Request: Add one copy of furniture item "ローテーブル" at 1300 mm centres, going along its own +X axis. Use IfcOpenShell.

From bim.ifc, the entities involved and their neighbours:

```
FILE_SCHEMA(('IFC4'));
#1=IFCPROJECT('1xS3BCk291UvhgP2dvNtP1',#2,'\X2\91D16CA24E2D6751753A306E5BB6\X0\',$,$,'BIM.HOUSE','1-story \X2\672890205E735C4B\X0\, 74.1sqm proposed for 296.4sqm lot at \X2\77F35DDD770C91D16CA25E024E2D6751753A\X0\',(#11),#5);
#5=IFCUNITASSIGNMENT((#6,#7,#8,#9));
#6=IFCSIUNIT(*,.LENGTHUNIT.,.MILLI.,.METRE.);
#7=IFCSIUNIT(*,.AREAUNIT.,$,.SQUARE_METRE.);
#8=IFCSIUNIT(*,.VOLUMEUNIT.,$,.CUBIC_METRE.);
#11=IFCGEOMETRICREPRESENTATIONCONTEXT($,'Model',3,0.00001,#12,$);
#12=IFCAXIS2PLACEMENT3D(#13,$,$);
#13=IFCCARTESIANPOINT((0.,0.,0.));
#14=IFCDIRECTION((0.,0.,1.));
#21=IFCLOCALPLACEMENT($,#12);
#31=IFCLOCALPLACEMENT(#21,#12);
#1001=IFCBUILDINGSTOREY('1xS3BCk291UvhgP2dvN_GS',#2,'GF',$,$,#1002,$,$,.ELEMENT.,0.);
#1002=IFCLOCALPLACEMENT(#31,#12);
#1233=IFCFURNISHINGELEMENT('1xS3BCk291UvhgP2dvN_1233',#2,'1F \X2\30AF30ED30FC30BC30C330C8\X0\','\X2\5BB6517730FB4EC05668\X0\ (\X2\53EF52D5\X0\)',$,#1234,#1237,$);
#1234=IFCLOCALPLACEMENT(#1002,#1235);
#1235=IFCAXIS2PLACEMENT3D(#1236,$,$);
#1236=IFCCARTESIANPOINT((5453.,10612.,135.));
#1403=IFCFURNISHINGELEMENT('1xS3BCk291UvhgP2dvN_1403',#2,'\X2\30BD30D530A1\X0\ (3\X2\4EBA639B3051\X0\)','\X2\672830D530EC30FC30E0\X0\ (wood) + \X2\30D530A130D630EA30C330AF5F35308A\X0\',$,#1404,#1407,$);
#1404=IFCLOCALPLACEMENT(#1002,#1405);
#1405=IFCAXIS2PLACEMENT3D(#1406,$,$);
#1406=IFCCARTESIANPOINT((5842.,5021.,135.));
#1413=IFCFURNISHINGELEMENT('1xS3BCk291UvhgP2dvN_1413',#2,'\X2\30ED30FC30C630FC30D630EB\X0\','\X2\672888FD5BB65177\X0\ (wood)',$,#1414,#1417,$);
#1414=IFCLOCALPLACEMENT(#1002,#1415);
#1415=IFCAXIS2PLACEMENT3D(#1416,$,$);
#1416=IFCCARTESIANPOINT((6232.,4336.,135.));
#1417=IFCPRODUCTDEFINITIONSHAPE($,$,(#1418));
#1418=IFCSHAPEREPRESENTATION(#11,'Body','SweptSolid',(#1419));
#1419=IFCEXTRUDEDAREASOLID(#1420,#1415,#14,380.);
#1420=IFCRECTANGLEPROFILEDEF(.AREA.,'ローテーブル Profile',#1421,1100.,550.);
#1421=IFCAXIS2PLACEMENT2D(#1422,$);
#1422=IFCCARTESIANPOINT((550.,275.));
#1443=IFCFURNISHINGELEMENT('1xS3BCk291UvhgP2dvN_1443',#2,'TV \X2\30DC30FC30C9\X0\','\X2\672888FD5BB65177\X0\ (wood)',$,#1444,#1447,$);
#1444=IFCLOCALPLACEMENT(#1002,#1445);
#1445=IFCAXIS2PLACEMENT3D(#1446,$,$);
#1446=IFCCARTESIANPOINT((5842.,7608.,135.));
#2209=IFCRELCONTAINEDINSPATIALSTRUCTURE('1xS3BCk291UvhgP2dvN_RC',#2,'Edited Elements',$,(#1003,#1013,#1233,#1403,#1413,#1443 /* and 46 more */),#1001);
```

```python
import ifcopenshell
import ifcopenshell.api.geometry
import ifcopenshell.api.root
import ifcopenshell.util.element
import ifcopenshell.util.placement
import ifcopenshell.util.unit

model = ifcopenshell.open("bim.ifc")
unit_scale = ifcopenshell.util.unit.calculate_unit_scale(model)


def reuse_history(source, copy):
    """copy_class also copies each property set's owner history, people and application; keep the originals."""
    for rel in copy.IsDefinedBy:
        if rel.is_a("IfcRelDefinesByProperties") and (history := rel.RelatingPropertyDefinition.OwnerHistory):
            rel.RelatingPropertyDefinition.OwnerHistory = source.OwnerHistory
            ifcopenshell.util.element.remove_deep2(model, history)


source = model.by_guid("1xS3BCk291UvhgP2dvN_1413")
base = ifcopenshell.util.placement.get_local_placement(source.ObjectPlacement)
step = base[:3, 0] * 1.3 / unit_scale

for i in range(1, 2):
    copy = ifcopenshell.api.root.copy_class(model, product=source)
    copy.Representation = ifcopenshell.util.element.copy_deep(
        model, source.Representation, exclude=["IfcGeometricRepresentationContext", "IfcRepresentationMap"]
    )
    reuse_history(source, copy)
    matrix = base.copy()
    matrix[:3, 3] += i * step
    print("added at", matrix[:3, 3].round(3) + 0.0)
    ifcopenshell.api.geometry.edit_object_placement(model, product=copy, matrix=matrix, is_si=False)

model.write("bim_rev.ifc")
```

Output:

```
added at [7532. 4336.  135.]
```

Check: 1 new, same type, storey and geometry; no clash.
